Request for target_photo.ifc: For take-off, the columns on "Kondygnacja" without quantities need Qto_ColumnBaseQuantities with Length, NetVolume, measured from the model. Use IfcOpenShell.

First a look at what the model holds.

```python
import ifcopenshell
import ifcopenshell.util.element
import ifcopenshell.util.unit

model = ifcopenshell.open("target_photo.ifc")
print(model.schema)
for unit_type in ("LENGTHUNIT", "AREAUNIT", "VOLUMEUNIT"):
    print(unit_type, ifcopenshell.util.unit.calculate_unit_scale(model, unit_type))
storey = next(s for s in model.by_type("IfcBuildingStorey") if s.Name == "Kondygnacja")
columns = [e for e in ifcopenshell.util.element.get_decomposition(storey) if e.is_a("IfcColumn")]
for e in sorted(columns, key=lambda e: e.id()):
    print(e.id(), e.is_a(), e.Name, list(ifcopenshell.util.element.get_psets(e, qtos_only=True)), sep=" | ")
```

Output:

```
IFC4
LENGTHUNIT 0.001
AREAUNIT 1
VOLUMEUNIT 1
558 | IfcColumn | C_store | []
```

```python
import ifcopenshell
import ifcopenshell.api.pset
import ifcopenshell.geom
import ifcopenshell.util.element
import ifcopenshell.util.shape
import ifcopenshell.util.unit

model = ifcopenshell.open("target_photo.ifc")
unit_scale = ifcopenshell.util.unit.calculate_unit_scale(model)
volume_scale = ifcopenshell.util.unit.calculate_unit_scale(model, "VOLUMEUNIT")
settings = ifcopenshell.geom.settings()

storey = next(s for s in model.by_type("IfcBuildingStorey") if s.Name == "Kondygnacja")
columns = [e for e in ifcopenshell.util.element.get_decomposition(storey) if e.is_a("IfcColumn")]

for e in sorted(columns, key=lambda e: e.id()):
    if ifcopenshell.util.element.get_psets(e, qtos_only=True, should_inherit=False):
        continue
    # Geometry comes back in metres, in the element's own axes.
    shape = ifcopenshell.geom.create_shape(settings, e)
    values = {
        "Length": ifcopenshell.util.shape.get_z(shape.geometry) / unit_scale,
        "NetVolume": ifcopenshell.util.shape.get_volume(shape.geometry) / volume_scale,
    }
    qto = ifcopenshell.api.pset.add_qto(model, product=e, name="Qto_ColumnBaseQuantities")
    ifcopenshell.api.pset.edit_qto(model, qto=qto, properties=values)
    print(e.id(), {k: round(v, 3) for k, v in values.items()})

model.write("target_photo_rev.ifc")
```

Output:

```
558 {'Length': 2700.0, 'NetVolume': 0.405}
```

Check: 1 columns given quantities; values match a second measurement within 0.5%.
